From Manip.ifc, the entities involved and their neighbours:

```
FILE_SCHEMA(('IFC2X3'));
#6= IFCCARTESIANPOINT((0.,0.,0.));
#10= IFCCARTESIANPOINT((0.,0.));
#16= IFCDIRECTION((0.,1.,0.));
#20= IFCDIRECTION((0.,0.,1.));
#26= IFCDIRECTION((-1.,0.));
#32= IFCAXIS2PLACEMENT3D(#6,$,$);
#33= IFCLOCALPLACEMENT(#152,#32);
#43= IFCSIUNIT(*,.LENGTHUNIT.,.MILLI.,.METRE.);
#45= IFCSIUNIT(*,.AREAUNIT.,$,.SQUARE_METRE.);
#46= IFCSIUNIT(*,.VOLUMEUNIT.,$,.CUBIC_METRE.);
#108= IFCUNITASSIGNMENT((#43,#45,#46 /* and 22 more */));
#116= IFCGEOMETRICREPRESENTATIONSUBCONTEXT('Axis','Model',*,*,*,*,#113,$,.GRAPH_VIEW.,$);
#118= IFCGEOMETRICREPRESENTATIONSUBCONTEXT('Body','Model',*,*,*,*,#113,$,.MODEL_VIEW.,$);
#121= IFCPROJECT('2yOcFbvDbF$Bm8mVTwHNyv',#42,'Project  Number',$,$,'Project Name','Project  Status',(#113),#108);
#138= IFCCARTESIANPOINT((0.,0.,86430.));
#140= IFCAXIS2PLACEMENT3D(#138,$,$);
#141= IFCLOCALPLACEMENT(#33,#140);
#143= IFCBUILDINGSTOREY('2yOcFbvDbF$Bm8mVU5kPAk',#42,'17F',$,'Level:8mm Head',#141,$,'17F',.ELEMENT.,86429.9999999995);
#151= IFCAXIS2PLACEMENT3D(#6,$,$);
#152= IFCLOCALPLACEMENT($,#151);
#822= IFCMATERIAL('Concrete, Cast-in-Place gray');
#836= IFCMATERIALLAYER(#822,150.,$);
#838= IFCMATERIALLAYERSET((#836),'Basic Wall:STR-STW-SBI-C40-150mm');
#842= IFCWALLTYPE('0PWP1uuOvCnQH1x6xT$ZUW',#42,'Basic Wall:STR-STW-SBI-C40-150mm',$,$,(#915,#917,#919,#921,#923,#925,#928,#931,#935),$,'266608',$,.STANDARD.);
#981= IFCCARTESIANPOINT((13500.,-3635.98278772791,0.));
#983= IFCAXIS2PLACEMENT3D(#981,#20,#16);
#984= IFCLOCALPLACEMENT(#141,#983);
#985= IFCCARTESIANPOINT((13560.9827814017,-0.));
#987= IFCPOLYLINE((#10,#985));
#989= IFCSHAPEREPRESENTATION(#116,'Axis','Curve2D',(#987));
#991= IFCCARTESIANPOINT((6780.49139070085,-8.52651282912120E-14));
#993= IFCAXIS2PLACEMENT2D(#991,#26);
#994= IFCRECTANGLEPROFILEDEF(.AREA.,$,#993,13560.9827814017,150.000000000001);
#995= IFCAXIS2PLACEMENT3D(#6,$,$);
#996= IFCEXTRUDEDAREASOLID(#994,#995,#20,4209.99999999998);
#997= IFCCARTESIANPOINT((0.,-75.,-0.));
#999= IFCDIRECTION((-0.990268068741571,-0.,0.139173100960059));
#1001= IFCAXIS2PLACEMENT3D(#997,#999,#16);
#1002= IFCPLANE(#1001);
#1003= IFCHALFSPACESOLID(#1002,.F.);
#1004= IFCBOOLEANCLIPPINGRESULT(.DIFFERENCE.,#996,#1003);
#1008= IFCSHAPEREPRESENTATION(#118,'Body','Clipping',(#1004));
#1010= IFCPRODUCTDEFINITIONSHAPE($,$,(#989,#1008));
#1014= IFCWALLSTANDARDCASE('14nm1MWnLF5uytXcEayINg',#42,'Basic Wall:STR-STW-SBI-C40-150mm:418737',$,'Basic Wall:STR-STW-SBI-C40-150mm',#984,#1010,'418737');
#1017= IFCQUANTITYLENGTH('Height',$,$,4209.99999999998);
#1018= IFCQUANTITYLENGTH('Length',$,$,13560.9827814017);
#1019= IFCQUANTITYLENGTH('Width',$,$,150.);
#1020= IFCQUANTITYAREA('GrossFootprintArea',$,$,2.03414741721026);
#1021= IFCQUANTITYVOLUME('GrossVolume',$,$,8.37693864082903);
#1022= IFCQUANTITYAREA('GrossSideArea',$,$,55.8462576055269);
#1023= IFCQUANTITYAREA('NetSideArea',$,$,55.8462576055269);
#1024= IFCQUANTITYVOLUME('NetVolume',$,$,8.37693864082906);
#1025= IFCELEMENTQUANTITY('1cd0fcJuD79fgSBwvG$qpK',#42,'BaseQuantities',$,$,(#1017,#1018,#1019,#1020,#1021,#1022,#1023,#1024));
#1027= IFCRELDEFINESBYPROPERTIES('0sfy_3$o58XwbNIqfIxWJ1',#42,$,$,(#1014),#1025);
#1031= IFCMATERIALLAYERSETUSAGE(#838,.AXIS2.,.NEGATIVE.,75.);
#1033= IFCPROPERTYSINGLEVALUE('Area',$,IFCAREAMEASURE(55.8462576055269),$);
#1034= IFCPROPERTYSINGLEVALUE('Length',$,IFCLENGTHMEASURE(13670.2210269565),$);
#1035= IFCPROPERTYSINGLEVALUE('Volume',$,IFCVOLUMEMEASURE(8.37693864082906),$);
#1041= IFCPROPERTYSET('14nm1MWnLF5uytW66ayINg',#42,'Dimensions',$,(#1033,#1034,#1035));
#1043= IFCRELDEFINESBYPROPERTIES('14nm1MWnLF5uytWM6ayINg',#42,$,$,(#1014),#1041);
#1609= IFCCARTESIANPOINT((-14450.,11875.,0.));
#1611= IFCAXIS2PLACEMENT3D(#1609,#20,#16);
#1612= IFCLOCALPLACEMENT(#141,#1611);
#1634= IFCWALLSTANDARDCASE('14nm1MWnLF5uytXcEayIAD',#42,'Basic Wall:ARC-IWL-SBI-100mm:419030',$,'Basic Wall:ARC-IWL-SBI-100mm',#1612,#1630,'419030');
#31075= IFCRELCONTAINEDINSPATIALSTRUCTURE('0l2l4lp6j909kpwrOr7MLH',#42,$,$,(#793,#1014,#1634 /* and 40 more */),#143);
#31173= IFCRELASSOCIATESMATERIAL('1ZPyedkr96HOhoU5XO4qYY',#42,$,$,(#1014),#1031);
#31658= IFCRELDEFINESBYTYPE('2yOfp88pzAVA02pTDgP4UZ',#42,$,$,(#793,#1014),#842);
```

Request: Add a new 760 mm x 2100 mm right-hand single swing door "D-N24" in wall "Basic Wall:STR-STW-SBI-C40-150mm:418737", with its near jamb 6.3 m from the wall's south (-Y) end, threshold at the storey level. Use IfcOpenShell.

```python
import numpy as np
import ifcopenshell
import ifcopenshell.api.feature
import ifcopenshell.api.geometry
import ifcopenshell.api.pset
import ifcopenshell.api.root
import ifcopenshell.api.spatial
import ifcopenshell.api.type
import ifcopenshell.geom
import ifcopenshell.util.element
import ifcopenshell.util.placement
import ifcopenshell.util.representation
import ifcopenshell.util.shape
import ifcopenshell.util.unit

model = ifcopenshell.open("Manip.ifc")
unit_scale = ifcopenshell.util.unit.calculate_unit_scale(model)
area_scale = ifcopenshell.util.unit.calculate_unit_scale(model, "AREAUNIT")
volume_scale = ifcopenshell.util.unit.calculate_unit_scale(model, "VOLUMEUNIT")
settings = ifcopenshell.geom.settings()


def volume(element):
    """Net volume in cubic metres, openings subtracted."""
    shape = ifcopenshell.geom.create_shape(settings, element)
    return ifcopenshell.util.shape.get_volume(shape.geometry)


wall = model.by_guid("14nm1MWnLF5uytXcEayINg")
storey = ifcopenshell.util.element.get_container(wall, ifc_class="IfcBuildingStorey")
context = ifcopenshell.util.representation.get_context(model, "Model", "Body", "MODEL_VIEW")
before = volume(wall)

width, height, from_end, sill = 0.76, 2.1, 6.3, 0.0  # metres

# The wall runs along its own X axis, and the end named is its -X end.
wall_shape = ifcopenshell.geom.create_shape(settings, wall)
x, y, z = ifcopenshell.util.shape.get_vertices(wall_shape.geometry).T
start = x.min() + from_end
face, thickness = float(y.min()), float(y.max() - y.min())
wall_matrix = ifcopenshell.util.placement.get_local_placement(wall.ObjectPlacement)
level = ifcopenshell.util.placement.get_local_placement(storey.ObjectPlacement)[2, 3]


def in_wall(x, y):
    """Placement at x, y metres in the wall's axes, at sill height."""
    matrix = wall_matrix.copy()
    matrix[:, 3] = wall_matrix @ np.array([x / unit_scale, y / unit_scale, 0.0, 1.0])
    matrix[2, 3] = level + sill / unit_scale
    return matrix


# Opening: a box that overshoots both wall faces by 50 mm.
opening = ifcopenshell.api.root.create_entity(model, ifc_class="IfcOpeningElement")
box = ifcopenshell.api.geometry.add_wall_representation(
    model, context=context, length=width, height=height, thickness=thickness + 0.1
)
ifcopenshell.api.geometry.assign_representation(model, product=opening, representation=box)
ifcopenshell.api.geometry.edit_object_placement(model, product=opening, matrix=in_wall(start, face - 0.05), is_si=False)
ifcopenshell.api.feature.add_feature(model, feature=opening, element=wall)

door = ifcopenshell.api.root.create_entity(model, ifc_class="IfcDoor", name="D-N24")
door.OverallWidth, door.OverallHeight = width / unit_scale, height / unit_scale
body = ifcopenshell.api.geometry.add_door_representation(
    model,
    context=context,
    overall_width=door.OverallWidth,
    overall_height=door.OverallHeight,
    operation_type="SINGLE_SWING_RIGHT",
    lining_properties={"LiningDepth": thickness / unit_scale, "ThresholdDepth": thickness / unit_scale},
)
ifcopenshell.api.geometry.assign_representation(model, product=door, representation=body)
ifcopenshell.api.spatial.assign_container(model, products=[door], relating_structure=storey)
fills = ifcopenshell.api.feature.add_filling(model, opening=opening, element=door)
fills.OwnerHistory = door.OwnerHistory  # required in IFC2X3

# IFC2X3 keeps the operation on the door style.
style = ifcopenshell.api.root.create_entity(model, ifc_class="IfcDoorStyle", name="D-N24")
style.OperationType, style.ConstructionType = "SINGLE_SWING_RIGHT", "NOTDEFINED"
style.ParameterTakesPrecedence = style.Sizeable = False
ifcopenshell.api.type.assign_type(model, related_objects=[door], relating_type=style)

# The lining spans the wall, so the door starts at the wall face.
ifcopenshell.api.geometry.edit_object_placement(model, product=door, matrix=in_wall(start, face), is_si=False)

after = volume(wall)

# Update the wall's stored quantities.
qto = model.by_id(ifcopenshell.util.element.get_pset(wall, "BaseQuantities", should_inherit=False)["id"])
ifcopenshell.api.pset.edit_qto(model, qto=qto, properties={
    "NetSideArea": after / thickness / area_scale,
    "NetVolume": after / volume_scale,
})
pset = model.by_id(ifcopenshell.util.element.get_pset(wall, "Dimensions", should_inherit=False)["id"])
ifcopenshell.api.pset.edit_pset(model, pset=pset, properties={
    "Area": model.create_entity("IfcAreaMeasure", after / thickness / area_scale),
    "Volume": model.create_entity("IfcVolumeMeasure", after / volume_scale),
})

print(f"wall volume {before:.3f} -> {after:.3f} m3")

model.write("Manip_v2.ifc")
```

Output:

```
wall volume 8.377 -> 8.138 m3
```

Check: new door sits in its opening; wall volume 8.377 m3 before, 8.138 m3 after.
